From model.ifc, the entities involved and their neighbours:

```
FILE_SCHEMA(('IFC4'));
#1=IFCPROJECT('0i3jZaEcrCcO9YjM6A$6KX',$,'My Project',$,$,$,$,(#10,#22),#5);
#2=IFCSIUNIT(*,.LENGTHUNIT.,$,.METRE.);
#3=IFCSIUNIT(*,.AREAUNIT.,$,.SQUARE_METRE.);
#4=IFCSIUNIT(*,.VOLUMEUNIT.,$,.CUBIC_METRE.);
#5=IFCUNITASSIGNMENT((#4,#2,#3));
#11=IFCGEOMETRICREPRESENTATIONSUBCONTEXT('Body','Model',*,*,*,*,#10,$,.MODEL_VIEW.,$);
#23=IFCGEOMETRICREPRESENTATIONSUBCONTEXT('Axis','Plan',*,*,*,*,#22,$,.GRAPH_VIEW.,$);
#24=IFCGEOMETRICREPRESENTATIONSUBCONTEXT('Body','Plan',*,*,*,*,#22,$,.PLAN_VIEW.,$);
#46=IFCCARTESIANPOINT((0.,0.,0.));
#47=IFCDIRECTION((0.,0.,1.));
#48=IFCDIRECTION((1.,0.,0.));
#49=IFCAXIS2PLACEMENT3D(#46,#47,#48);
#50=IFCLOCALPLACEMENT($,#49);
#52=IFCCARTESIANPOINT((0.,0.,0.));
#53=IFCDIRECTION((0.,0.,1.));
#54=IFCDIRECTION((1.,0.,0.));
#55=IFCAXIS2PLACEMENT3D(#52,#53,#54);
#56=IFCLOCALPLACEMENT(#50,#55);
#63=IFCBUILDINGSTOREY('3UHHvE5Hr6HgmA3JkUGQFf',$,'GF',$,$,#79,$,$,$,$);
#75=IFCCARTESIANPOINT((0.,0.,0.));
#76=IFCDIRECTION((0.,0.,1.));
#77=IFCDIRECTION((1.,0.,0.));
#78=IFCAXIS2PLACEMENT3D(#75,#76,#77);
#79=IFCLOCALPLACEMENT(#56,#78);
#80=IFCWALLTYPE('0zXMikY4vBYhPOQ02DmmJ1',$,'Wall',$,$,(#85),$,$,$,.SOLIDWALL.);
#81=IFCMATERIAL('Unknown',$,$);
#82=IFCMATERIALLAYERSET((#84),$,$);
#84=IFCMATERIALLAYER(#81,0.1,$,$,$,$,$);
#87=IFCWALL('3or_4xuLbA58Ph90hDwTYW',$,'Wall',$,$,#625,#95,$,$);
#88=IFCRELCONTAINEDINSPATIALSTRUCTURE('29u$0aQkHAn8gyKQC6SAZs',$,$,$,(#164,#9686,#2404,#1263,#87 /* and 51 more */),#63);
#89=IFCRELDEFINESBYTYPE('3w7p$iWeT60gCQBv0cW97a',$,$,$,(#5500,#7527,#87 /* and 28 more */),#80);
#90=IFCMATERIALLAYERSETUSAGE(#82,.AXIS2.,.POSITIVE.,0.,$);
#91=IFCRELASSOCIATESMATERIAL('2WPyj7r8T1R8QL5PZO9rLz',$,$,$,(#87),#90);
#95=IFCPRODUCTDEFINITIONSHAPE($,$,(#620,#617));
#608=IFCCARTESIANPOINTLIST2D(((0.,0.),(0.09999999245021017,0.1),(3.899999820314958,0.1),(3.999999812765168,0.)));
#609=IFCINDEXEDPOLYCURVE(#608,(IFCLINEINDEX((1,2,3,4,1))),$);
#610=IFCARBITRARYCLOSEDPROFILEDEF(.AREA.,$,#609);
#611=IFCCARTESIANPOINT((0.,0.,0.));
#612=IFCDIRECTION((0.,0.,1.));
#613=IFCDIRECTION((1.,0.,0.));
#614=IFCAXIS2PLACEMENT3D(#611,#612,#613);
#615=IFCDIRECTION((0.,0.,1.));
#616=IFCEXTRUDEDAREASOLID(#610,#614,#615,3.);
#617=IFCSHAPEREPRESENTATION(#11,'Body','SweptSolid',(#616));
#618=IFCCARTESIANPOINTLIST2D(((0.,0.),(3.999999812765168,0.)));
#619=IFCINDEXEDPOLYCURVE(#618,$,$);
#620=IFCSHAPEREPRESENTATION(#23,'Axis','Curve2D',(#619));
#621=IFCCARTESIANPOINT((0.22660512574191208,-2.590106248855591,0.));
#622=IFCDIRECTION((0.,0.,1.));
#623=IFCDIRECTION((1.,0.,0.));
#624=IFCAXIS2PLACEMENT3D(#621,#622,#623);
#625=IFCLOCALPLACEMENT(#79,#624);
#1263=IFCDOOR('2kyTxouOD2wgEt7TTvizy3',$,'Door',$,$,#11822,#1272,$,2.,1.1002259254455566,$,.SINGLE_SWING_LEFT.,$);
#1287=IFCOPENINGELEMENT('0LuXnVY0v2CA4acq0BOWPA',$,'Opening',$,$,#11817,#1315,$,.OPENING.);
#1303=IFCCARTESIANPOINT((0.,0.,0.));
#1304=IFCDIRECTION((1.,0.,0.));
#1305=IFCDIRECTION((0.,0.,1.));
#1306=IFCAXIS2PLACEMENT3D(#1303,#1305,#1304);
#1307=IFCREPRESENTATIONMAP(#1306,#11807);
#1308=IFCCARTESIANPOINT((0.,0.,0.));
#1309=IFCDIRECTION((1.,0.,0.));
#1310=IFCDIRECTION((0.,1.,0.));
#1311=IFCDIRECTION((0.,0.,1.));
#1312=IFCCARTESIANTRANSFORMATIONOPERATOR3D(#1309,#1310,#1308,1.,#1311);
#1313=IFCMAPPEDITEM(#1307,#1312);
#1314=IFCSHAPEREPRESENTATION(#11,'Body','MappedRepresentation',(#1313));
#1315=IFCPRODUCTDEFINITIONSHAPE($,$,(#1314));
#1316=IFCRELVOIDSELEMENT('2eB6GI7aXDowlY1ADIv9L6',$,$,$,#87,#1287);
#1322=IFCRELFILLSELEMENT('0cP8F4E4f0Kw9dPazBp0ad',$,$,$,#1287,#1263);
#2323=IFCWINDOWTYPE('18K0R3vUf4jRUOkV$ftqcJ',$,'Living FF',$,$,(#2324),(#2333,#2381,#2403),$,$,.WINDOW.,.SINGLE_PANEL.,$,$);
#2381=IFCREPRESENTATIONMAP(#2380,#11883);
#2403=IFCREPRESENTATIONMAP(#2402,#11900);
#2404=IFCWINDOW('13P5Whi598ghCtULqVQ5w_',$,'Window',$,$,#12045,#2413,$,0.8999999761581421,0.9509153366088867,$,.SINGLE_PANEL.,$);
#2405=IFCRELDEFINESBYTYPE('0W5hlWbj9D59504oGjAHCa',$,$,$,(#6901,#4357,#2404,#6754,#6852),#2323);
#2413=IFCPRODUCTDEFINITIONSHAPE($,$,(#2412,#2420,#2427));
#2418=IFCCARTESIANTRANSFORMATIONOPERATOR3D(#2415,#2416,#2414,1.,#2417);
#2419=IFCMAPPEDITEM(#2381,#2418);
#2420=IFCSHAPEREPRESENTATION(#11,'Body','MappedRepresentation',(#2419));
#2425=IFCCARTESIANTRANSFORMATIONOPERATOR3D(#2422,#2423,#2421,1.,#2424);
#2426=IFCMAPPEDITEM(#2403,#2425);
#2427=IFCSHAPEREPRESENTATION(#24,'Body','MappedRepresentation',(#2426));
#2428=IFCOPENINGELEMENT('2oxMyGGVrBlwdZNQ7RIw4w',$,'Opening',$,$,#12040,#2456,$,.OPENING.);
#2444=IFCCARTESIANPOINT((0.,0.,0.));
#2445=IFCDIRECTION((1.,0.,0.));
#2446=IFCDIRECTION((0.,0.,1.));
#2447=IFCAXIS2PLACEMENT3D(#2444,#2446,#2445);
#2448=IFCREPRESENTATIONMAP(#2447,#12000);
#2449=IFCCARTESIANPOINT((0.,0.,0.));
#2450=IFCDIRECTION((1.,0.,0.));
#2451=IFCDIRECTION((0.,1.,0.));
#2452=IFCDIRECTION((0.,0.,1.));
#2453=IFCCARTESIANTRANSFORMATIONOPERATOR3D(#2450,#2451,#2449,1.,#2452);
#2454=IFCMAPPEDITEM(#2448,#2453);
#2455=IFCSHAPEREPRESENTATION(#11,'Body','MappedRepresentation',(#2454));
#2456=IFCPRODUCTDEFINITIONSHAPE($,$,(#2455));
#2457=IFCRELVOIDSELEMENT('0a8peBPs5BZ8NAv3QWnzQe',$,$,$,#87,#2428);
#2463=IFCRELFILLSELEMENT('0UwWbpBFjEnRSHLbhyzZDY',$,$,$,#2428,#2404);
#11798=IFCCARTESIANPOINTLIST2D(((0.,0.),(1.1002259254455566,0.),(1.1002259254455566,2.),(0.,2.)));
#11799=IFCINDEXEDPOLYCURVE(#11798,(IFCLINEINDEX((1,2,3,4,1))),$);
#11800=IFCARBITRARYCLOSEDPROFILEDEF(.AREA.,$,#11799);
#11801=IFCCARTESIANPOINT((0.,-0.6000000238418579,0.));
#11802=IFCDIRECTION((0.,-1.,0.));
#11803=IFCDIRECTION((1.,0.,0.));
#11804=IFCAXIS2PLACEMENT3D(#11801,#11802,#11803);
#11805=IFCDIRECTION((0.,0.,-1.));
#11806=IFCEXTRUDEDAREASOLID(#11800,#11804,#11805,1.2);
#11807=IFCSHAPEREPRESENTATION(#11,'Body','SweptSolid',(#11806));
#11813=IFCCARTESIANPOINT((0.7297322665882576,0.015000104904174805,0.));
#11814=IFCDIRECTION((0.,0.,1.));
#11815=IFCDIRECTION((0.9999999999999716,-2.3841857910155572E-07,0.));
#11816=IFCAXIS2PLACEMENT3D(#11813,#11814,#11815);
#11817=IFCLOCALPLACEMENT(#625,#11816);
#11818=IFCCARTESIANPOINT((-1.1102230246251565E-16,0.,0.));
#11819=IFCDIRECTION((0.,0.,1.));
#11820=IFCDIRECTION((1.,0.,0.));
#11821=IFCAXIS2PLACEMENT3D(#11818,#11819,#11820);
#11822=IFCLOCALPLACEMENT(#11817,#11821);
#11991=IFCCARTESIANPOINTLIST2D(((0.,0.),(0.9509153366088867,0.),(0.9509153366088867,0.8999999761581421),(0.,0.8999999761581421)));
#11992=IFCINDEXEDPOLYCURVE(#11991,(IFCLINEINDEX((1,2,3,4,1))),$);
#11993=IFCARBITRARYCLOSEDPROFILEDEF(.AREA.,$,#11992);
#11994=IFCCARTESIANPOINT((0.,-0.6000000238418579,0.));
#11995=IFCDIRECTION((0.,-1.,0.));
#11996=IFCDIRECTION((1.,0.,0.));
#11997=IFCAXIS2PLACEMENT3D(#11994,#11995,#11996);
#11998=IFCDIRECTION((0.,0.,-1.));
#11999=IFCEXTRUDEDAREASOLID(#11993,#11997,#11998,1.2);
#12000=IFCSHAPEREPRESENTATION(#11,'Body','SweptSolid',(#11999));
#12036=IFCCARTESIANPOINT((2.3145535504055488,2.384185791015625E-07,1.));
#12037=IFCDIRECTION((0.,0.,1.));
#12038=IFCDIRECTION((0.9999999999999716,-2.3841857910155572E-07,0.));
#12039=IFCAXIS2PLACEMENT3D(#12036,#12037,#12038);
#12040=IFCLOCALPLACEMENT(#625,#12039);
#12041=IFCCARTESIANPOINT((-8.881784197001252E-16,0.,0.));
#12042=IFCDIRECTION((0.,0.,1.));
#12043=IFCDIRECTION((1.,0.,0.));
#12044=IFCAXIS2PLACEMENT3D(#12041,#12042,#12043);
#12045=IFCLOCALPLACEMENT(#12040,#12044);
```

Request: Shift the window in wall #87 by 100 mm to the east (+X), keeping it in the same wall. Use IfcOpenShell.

```python
import ifcopenshell
import ifcopenshell.api.geometry
import ifcopenshell.util.placement

model = ifcopenshell.open("model.ifc")

window = model.by_guid("13P5Whi598ghCtULqVQ5w_")
opening = window.FillsVoids[0].RelatingOpeningElement
wall = opening.VoidsElements[0].RelatingBuildingElement

wall_matrix = ifcopenshell.util.placement.get_local_placement(wall.ObjectPlacement)
shift = wall_matrix[:3, 0] * 0.1
before = ifcopenshell.util.placement.get_local_placement(window.ObjectPlacement)[:3, 3].copy()

# The window is placed relative to its opening, so it follows when the opening moves.
matrix = ifcopenshell.util.placement.get_local_placement(opening.ObjectPlacement)
matrix[:3, 3] += shift
ifcopenshell.api.geometry.edit_object_placement(
    model, product=opening, matrix=matrix, is_si=False, should_transform_children=True
)

after = ifcopenshell.util.placement.get_local_placement(window.ObjectPlacement)[:3, 3]
print("window moved by", (after - before).round(3) + 0.0)

model.write("model-out.ifc")
```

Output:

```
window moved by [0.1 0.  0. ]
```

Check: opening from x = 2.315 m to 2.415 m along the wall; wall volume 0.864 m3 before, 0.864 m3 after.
